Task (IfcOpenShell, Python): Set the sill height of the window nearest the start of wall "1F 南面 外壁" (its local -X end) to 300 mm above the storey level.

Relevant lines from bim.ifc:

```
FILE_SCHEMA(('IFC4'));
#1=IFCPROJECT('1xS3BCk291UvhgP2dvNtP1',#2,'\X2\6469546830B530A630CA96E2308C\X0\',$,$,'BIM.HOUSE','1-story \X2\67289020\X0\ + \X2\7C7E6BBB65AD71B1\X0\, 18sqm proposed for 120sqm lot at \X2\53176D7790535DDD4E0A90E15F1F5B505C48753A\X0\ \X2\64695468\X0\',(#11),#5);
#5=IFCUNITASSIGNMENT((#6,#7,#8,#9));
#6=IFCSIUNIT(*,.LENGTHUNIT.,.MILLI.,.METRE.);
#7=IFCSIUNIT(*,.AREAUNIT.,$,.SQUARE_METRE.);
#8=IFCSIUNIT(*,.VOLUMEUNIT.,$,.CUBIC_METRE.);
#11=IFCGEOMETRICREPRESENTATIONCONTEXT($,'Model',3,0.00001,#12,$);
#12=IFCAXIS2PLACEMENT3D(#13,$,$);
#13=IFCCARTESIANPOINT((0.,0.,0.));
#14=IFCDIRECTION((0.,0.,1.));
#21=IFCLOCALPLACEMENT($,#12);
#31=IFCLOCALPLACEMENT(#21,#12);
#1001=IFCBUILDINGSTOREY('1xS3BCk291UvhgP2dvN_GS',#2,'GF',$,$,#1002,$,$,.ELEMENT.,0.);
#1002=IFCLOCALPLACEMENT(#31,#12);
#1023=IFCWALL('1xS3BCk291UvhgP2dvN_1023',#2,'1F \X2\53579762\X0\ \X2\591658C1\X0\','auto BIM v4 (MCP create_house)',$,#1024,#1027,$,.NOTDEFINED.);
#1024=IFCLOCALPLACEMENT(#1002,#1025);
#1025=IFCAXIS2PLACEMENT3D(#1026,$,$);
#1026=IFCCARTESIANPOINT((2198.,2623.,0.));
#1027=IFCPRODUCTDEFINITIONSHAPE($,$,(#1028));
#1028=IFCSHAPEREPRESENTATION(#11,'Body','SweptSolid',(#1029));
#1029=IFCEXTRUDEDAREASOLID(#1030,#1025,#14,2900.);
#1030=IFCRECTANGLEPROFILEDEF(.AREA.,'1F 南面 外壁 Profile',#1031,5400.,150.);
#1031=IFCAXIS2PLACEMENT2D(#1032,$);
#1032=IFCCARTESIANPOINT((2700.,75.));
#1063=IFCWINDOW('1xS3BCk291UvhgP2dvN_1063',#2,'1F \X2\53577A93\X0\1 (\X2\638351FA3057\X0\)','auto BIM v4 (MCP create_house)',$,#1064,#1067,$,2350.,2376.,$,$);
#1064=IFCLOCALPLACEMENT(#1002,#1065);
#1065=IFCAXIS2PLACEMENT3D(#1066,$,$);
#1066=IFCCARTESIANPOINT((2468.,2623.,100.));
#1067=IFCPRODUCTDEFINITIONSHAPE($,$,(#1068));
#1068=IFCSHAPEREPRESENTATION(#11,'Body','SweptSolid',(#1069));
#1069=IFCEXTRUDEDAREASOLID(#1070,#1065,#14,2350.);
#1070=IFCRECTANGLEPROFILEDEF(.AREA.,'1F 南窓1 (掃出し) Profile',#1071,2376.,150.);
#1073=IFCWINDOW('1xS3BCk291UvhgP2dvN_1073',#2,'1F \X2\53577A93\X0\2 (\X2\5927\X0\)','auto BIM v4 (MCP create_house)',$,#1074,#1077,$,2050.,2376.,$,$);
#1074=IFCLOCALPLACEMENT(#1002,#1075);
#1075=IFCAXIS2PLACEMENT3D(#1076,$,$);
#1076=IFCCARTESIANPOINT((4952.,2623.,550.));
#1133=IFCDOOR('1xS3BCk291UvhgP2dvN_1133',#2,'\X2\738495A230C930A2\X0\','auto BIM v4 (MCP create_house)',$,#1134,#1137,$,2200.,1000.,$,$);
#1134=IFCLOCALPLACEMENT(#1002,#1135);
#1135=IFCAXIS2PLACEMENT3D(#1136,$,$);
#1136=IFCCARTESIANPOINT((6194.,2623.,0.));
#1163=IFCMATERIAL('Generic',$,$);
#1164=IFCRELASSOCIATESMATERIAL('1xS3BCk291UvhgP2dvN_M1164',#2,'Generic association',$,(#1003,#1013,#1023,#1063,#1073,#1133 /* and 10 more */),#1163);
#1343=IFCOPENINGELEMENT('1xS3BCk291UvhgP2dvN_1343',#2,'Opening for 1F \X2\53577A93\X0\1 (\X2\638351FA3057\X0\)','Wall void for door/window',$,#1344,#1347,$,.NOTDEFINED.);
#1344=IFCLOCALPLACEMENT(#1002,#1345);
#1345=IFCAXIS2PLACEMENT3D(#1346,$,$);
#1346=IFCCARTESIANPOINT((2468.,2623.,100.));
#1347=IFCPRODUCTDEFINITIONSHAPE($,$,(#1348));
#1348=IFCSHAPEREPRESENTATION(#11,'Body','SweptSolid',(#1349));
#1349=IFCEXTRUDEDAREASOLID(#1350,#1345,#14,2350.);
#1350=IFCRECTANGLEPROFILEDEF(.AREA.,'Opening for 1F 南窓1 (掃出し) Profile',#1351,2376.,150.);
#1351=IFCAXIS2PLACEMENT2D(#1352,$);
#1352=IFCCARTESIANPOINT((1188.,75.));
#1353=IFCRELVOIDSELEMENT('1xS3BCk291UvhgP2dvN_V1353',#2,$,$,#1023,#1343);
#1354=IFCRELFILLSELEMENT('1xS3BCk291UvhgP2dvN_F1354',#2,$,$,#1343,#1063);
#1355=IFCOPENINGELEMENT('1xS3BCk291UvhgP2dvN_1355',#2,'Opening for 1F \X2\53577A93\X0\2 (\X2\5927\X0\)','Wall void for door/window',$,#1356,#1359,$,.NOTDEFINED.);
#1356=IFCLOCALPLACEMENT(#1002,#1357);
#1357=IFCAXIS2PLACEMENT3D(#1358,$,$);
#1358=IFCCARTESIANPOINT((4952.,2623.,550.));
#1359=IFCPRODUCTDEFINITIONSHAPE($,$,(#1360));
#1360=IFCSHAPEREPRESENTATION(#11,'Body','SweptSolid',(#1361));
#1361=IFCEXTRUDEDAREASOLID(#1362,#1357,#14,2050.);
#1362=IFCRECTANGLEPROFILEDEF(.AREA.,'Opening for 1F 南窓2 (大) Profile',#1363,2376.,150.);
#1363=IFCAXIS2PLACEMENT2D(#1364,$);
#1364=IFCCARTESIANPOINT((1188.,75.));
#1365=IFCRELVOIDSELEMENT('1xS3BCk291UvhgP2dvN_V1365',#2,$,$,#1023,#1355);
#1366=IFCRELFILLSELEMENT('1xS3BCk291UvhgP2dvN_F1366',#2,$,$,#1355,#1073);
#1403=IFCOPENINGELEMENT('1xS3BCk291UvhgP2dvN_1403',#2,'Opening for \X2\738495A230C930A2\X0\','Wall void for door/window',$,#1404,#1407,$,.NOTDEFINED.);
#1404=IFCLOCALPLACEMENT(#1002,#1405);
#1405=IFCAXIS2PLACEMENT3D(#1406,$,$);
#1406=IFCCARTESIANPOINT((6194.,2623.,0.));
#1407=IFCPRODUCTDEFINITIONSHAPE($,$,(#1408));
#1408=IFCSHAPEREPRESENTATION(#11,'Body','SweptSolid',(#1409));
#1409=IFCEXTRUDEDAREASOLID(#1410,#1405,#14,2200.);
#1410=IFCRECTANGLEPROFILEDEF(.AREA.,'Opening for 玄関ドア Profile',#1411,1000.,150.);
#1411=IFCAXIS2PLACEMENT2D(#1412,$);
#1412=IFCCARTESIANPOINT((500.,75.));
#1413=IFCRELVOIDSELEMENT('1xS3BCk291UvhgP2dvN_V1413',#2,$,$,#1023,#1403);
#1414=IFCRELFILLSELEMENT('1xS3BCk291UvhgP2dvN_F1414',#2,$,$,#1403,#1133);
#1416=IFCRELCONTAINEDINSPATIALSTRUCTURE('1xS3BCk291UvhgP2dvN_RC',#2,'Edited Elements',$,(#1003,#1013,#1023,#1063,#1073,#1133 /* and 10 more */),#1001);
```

```python
import numpy as np
import ifcopenshell
import ifcopenshell.api.geometry
import ifcopenshell.geom
import ifcopenshell.util.element
import ifcopenshell.util.placement
import ifcopenshell.util.shape
import ifcopenshell.util.unit

model = ifcopenshell.open("bim.ifc")
unit_scale = ifcopenshell.util.unit.calculate_unit_scale(model)

window = model.by_id(1063)
opening = window.FillsVoids[0].RelatingOpeningElement
storey = ifcopenshell.util.element.get_container(window, ifc_class="IfcBuildingStorey")
level = ifcopenshell.util.placement.get_local_placement(storey.ObjectPlacement)[2, 3]

# The opening's origin need not be at the sill, so measure its lowest point.
shape = ifcopenshell.geom.create_shape(ifcopenshell.geom.settings(), opening)
bottom = ifcopenshell.util.shape.get_shape_bottom_elevation(shape, shape.geometry) / unit_scale
dz = level + 300.0 - bottom

shift = np.array([0.0, 0.0, dz])
# The window is not placed relative to its opening, so move both.
for product in (opening, window):
    matrix = ifcopenshell.util.placement.get_local_placement(product.ObjectPlacement)
    matrix[:3, 3] += shift
    ifcopenshell.api.geometry.edit_object_placement(model, product=product, matrix=matrix, is_si=False)

print(f"moved by {dz * unit_scale:+.3f} m")

model.write("bim_rev.ifc")
```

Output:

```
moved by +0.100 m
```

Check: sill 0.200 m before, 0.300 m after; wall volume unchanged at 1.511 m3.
